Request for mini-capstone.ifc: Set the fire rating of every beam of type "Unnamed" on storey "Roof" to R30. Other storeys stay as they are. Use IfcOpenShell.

First a look at what the model holds.

```python
import ifcopenshell
import ifcopenshell.util.element

model = ifcopenshell.open("mini-capstone.ifc")
print(model.schema)
storey = next(s for s in model.by_type("IfcBuildingStorey") if s.Name == "Roof")
beams = [e for e in ifcopenshell.util.element.get_decomposition(storey) if e.is_a("IfcBeam")]
seen = {}
for e in beams:
    element_type = ifcopenshell.util.element.get_type(e)
    key = (element_type.Name if element_type != e and element_type else None, ifcopenshell.util.element.get_pset(e, "Pset_BeamCommon", "FireRating"))
    seen[key] = seen.get(key, 0) + 1
for (name, value), count in sorted(seen.items(), key=str):
    print(count, "x", name, "|", value)
```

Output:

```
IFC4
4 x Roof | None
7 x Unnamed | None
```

```python
import ifcopenshell
import ifcopenshell.api.pset
import ifcopenshell.util.element

model = ifcopenshell.open("mini-capstone.ifc")

storey = next(s for s in model.by_type("IfcBuildingStorey") if s.Name == "Roof")
beams = [e for e in ifcopenshell.util.element.get_decomposition(storey) if e.is_a("IfcBeam")]

count = 0
for e in beams:
    element_type = ifcopenshell.util.element.get_type(e)
    if element_type in (None, e) or element_type.Name != "Unnamed":
        continue
    # add_pset returns the element's existing set when there is one.
    pset = ifcopenshell.api.pset.add_pset(model, product=e, name="Pset_BeamCommon")
    ifcopenshell.api.pset.edit_pset(model, pset=pset, properties={"FireRating": "R30"})
    count += 1

print(count, "beams updated")

model.write("mini-capstone_v2.ifc")
```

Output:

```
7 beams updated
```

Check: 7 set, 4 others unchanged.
